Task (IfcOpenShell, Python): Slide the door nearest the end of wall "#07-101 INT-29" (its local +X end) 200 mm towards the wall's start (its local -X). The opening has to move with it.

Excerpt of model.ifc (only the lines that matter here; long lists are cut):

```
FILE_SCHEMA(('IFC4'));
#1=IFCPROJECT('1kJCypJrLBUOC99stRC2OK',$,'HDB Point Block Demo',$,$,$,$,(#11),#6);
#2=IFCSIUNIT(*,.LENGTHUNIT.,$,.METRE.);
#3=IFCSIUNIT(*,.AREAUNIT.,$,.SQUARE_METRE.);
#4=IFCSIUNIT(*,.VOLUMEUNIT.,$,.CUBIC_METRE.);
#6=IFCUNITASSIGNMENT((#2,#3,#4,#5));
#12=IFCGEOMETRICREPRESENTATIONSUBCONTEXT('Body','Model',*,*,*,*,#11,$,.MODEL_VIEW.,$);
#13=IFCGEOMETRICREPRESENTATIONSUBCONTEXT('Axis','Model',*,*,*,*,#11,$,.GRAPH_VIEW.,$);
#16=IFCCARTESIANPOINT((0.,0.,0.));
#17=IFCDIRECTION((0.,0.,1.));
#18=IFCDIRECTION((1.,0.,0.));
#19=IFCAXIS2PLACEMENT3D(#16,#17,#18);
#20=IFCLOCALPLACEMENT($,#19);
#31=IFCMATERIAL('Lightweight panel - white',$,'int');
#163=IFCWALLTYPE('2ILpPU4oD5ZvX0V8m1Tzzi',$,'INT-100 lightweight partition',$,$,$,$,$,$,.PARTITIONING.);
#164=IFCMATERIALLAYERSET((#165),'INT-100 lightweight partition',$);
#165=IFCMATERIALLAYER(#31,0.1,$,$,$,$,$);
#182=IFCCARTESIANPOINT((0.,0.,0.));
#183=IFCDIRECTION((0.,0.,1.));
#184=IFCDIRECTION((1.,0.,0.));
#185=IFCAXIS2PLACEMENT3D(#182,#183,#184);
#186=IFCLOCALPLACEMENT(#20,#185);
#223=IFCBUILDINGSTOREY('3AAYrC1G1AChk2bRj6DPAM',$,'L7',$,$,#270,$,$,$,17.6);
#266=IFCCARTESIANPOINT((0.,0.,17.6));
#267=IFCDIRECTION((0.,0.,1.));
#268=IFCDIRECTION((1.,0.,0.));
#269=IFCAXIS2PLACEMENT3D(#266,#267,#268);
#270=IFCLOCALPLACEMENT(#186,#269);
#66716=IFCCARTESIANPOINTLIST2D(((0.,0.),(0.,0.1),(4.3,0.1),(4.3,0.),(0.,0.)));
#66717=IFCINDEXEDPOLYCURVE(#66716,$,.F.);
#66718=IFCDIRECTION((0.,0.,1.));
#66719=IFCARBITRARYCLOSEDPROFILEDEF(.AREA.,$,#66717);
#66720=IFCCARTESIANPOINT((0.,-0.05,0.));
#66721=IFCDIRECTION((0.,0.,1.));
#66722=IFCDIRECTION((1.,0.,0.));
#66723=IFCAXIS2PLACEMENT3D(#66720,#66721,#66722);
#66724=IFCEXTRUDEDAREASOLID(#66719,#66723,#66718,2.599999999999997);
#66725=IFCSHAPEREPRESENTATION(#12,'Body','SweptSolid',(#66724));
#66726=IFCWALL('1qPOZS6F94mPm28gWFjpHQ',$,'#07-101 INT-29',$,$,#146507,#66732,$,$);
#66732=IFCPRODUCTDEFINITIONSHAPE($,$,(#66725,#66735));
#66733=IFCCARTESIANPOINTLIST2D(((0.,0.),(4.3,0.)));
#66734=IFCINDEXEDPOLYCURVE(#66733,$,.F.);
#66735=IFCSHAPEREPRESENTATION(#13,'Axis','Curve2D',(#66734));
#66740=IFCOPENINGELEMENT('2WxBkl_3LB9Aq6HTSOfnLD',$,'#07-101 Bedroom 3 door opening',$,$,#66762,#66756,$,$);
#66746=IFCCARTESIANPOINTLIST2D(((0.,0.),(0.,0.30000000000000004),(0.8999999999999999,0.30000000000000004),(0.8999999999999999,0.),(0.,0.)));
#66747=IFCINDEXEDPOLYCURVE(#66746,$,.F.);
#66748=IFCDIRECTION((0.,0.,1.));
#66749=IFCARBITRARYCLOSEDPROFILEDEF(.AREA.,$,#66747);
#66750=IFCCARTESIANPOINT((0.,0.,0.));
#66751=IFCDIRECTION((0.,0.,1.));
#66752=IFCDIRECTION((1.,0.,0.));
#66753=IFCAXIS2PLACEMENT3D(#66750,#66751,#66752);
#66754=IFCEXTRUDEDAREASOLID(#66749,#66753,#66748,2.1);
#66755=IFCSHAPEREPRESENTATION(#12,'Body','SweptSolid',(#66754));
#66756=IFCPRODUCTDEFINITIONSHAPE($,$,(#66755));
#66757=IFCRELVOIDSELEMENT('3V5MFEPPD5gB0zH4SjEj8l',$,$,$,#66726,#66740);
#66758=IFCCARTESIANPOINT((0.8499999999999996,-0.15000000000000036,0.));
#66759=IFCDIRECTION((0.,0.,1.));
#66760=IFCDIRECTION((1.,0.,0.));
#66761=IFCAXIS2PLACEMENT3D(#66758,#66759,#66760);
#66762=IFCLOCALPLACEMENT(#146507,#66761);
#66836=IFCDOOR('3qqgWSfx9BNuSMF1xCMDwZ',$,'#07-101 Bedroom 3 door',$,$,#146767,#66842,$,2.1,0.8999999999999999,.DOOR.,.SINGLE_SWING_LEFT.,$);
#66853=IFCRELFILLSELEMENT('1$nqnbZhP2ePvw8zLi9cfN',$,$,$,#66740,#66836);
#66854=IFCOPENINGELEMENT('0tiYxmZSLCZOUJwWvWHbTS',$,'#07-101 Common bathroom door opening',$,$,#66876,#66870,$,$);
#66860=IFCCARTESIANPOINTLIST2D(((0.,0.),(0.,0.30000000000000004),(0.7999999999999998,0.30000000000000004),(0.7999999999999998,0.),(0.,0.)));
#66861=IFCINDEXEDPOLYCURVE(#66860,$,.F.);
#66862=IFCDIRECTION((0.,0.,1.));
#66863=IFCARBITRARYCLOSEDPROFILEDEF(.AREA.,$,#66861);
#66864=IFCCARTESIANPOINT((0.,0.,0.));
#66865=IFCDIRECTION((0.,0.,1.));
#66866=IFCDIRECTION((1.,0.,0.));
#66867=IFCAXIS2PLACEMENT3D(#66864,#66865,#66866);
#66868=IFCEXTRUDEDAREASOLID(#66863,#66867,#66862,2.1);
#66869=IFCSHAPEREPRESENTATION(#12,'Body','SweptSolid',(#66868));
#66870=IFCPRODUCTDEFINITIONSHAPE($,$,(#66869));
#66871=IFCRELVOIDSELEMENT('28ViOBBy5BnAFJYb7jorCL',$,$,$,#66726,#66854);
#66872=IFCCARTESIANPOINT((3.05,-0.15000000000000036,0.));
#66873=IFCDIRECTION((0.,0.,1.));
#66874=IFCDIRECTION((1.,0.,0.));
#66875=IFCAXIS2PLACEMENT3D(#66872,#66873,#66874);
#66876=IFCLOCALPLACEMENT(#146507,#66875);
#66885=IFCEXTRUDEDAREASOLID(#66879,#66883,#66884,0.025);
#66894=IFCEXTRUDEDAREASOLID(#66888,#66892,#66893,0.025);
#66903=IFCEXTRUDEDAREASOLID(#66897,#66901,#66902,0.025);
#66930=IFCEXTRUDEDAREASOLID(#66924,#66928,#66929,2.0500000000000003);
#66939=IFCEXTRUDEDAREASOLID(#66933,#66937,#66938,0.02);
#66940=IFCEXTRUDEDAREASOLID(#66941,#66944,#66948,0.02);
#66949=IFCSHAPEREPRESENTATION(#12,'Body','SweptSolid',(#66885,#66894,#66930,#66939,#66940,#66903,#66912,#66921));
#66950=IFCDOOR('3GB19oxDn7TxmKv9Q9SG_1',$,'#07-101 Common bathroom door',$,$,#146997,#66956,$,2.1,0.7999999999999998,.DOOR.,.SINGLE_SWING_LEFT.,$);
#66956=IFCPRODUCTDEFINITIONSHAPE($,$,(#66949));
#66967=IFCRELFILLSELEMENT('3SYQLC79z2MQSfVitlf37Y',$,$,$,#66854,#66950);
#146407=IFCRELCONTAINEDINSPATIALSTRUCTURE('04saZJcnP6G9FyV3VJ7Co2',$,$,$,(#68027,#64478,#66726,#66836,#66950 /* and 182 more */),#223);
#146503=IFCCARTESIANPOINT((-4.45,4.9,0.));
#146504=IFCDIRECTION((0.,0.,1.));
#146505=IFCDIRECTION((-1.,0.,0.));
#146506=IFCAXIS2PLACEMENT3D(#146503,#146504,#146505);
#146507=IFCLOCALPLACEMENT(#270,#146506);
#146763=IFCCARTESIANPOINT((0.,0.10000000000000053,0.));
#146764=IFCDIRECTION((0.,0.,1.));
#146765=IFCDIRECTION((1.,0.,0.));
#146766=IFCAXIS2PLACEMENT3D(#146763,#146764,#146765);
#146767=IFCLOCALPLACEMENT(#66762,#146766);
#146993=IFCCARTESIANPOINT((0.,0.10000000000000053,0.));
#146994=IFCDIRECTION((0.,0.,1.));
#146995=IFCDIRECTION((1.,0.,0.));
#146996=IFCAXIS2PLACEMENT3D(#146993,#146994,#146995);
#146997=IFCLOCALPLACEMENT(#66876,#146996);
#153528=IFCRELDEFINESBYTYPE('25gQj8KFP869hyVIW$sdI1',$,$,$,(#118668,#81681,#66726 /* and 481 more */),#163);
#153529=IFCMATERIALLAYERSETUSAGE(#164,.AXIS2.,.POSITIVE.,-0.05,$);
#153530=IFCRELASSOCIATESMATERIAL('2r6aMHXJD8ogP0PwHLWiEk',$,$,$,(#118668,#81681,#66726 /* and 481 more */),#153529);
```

```python
import ifcopenshell
import ifcopenshell.api.geometry
import ifcopenshell.util.placement

model = ifcopenshell.open("model.ifc")

door = model.by_guid("3GB19oxDn7TxmKv9Q9SG_1")
opening = door.FillsVoids[0].RelatingOpeningElement
wall = opening.VoidsElements[0].RelatingBuildingElement

wall_matrix = ifcopenshell.util.placement.get_local_placement(wall.ObjectPlacement)
shift = wall_matrix[:3, 0] * -0.2
before = ifcopenshell.util.placement.get_local_placement(door.ObjectPlacement)[:3, 3].copy()

# The door is placed relative to its opening, so it follows when the opening moves.
matrix = ifcopenshell.util.placement.get_local_placement(opening.ObjectPlacement)
matrix[:3, 3] += shift
ifcopenshell.api.geometry.edit_object_placement(
    model, product=opening, matrix=matrix, is_si=False, should_transform_children=True
)

after = ifcopenshell.util.placement.get_local_placement(door.ObjectPlacement)[:3, 3]
print("door moved by", (after - before).round(3) + 0.0)

model.write("model_rev.ifc")
```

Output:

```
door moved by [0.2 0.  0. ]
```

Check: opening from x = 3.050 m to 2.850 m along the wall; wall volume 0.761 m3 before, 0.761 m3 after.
